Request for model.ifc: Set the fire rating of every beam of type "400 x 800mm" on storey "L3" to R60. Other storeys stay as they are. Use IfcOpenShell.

First a look at what the model holds.

```python
import ifcopenshell
import ifcopenshell.util.element

model = ifcopenshell.open("model.ifc")
print(model.schema)
storey = next(s for s in model.by_type("IfcBuildingStorey") if s.Name == "L3")
beams = [e for e in ifcopenshell.util.element.get_decomposition(storey) if e.is_a("IfcBeam")]
seen = {}
for e in beams:
    element_type = ifcopenshell.util.element.get_type(e)
    key = (element_type.Name if element_type != e and element_type else None, ifcopenshell.util.element.get_pset(e, "Pset_BeamCommon", "FireRating"))
    seen[key] = seen.get(key, 0) + 1
for (name, value), count in sorted(seen.items(), key=str):
    print(count, "x", name, "|", value)
```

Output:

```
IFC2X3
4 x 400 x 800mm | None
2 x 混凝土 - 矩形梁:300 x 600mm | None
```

```python
import ifcopenshell
import ifcopenshell.api.pset
import ifcopenshell.util.element

model = ifcopenshell.open("model.ifc")

storey = next(s for s in model.by_type("IfcBuildingStorey") if s.Name == "L3")
beams = [e for e in ifcopenshell.util.element.get_decomposition(storey) if e.is_a("IfcBeam")]

count = 0
for e in beams:
    element_type = ifcopenshell.util.element.get_type(e)
    if element_type in (None, e) or element_type.Name != "400 x 800mm":
        continue
    # add_pset returns the element's existing set when there is one.
    pset = ifcopenshell.api.pset.add_pset(model, product=e, name="Pset_BeamCommon")
    ifcopenshell.api.pset.edit_pset(model, pset=pset, properties={"FireRating": "R60"})
    count += 1

print(count, "beams updated")

model.write("model-out.ifc")
```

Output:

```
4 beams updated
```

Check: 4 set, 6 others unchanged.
